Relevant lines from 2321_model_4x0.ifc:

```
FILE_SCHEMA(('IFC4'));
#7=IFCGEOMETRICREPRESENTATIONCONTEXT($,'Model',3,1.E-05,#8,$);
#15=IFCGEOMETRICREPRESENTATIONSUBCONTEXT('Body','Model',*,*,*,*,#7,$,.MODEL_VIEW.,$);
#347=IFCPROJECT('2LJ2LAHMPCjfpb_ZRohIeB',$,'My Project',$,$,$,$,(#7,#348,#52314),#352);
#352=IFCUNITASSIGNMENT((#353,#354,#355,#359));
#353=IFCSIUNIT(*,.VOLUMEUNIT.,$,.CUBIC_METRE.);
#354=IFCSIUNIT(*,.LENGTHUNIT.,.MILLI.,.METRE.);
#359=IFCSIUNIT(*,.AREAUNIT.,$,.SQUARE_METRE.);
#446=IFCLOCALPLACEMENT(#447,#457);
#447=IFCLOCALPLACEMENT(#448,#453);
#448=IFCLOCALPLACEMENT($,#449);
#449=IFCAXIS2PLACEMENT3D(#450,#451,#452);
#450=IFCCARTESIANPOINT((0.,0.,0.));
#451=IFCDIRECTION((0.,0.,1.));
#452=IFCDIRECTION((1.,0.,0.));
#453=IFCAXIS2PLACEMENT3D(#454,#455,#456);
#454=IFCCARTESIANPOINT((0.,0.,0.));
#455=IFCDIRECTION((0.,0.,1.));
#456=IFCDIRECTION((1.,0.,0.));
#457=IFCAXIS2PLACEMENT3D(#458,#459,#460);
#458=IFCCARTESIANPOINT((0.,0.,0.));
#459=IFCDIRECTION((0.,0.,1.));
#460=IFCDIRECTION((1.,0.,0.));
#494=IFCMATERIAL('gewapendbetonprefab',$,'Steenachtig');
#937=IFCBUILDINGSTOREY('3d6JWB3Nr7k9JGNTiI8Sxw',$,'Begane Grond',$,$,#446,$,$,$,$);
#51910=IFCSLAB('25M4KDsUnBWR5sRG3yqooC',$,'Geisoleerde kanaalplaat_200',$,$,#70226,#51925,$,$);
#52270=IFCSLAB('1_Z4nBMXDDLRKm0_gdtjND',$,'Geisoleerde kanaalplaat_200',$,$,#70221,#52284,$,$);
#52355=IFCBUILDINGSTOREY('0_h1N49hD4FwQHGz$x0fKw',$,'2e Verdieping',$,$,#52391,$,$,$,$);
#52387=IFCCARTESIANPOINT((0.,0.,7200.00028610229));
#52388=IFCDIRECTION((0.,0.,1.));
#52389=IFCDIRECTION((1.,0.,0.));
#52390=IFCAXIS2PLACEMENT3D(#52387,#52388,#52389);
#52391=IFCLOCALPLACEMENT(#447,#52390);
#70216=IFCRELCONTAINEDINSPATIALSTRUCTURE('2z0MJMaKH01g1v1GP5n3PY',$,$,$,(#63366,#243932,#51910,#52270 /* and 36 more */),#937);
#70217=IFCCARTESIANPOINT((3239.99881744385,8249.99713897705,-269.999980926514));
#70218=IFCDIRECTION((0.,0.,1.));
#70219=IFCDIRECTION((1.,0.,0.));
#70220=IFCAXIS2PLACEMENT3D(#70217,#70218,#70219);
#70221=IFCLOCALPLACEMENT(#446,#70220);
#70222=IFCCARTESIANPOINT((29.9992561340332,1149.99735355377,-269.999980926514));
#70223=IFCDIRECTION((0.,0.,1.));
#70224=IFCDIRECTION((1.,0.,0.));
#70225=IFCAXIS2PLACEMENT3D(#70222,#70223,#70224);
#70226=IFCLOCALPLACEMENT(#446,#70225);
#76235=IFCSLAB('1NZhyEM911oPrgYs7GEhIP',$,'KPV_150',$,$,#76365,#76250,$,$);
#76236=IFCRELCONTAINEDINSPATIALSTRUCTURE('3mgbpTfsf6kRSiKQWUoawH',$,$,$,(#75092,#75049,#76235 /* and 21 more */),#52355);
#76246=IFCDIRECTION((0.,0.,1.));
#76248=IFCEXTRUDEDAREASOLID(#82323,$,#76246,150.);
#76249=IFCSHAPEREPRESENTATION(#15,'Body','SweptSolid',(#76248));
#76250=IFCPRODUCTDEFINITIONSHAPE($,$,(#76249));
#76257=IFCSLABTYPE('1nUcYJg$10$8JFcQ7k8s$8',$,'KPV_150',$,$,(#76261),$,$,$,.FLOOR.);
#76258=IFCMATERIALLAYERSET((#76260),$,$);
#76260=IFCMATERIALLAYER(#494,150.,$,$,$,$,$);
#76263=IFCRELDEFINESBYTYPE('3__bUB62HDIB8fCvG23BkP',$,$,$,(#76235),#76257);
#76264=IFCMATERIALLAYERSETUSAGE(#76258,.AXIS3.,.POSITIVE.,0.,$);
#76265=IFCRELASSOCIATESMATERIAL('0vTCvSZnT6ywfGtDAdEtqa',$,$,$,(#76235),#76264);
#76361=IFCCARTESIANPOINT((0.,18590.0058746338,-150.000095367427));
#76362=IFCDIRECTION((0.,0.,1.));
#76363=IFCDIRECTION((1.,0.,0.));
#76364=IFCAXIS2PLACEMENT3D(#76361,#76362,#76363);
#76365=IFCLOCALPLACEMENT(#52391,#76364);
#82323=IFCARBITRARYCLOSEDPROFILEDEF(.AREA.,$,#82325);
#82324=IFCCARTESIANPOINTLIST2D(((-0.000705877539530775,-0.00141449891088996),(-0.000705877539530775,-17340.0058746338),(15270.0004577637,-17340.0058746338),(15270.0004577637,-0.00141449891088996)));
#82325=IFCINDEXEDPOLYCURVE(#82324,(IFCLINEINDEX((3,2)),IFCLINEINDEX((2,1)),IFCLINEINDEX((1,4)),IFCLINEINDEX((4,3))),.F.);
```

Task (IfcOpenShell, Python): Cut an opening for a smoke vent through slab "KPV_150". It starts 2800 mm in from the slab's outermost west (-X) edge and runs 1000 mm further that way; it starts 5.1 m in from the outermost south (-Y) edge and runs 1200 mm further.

```python
import numpy as np
import ifcopenshell
import ifcopenshell.api.feature
import ifcopenshell.api.geometry
import ifcopenshell.api.root
import ifcopenshell.geom
import ifcopenshell.util.placement
import ifcopenshell.util.representation
import ifcopenshell.util.shape
import ifcopenshell.util.unit

model = ifcopenshell.open("2321_model_4x0.ifc")
unit_scale = ifcopenshell.util.unit.calculate_unit_scale(model)
settings = ifcopenshell.geom.settings()


def volume(element):
    """Net volume in cubic metres, openings subtracted."""
    shape = ifcopenshell.geom.create_shape(settings, element)
    return ifcopenshell.util.shape.get_volume(shape.geometry)


slab = model.by_guid("1NZhyEM911oPrgYs7GEhIP")
before = volume(slab)

# Extent in the slab's own axes, in metres. The edges named are its -X and -Y sides.
slab_shape = ifcopenshell.geom.create_shape(settings, slab)
vertices = ifcopenshell.util.shape.get_vertices(slab_shape.geometry)
x_min, y_min, bottom = vertices.min(axis=0)
top = vertices[:, 2].max()

opening = ifcopenshell.api.root.create_entity(model, ifc_class="IfcOpeningElement", name="Smoke vent opening", predefined_type="OPENING")
context = ifcopenshell.util.representation.get_context(model, "Model", "Body", "MODEL_VIEW")
width, depth = 1, 1.2
outline = [(0.0, 0.0), (width, 0.0), (width, depth), (0.0, depth), (0.0, 0.0)]
# Overshoot both faces by 50 mm so the cut is clean.
shape = ifcopenshell.api.geometry.add_slab_representation(
    model, context=context, depth=top - bottom + 0.1, polyline=outline
)
ifcopenshell.api.geometry.assign_representation(model, product=opening, representation=shape)

matrix = ifcopenshell.util.placement.get_local_placement(slab.ObjectPlacement)
matrix[:, 3] = matrix @ np.append(np.array([x_min + 2.8, y_min + 5.1, bottom - 0.05]) / unit_scale, 1.0)
ifcopenshell.api.geometry.edit_object_placement(model, product=opening, matrix=matrix, is_si=False)
ifcopenshell.api.feature.add_feature(model, feature=opening, element=slab)

after = volume(slab)

print(f"slab volume {before:.3f} -> {after:.3f} m3")

model.write("2321_model_4x0_edited.ifc")
```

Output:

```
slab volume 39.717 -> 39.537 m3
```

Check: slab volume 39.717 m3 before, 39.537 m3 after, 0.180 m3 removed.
